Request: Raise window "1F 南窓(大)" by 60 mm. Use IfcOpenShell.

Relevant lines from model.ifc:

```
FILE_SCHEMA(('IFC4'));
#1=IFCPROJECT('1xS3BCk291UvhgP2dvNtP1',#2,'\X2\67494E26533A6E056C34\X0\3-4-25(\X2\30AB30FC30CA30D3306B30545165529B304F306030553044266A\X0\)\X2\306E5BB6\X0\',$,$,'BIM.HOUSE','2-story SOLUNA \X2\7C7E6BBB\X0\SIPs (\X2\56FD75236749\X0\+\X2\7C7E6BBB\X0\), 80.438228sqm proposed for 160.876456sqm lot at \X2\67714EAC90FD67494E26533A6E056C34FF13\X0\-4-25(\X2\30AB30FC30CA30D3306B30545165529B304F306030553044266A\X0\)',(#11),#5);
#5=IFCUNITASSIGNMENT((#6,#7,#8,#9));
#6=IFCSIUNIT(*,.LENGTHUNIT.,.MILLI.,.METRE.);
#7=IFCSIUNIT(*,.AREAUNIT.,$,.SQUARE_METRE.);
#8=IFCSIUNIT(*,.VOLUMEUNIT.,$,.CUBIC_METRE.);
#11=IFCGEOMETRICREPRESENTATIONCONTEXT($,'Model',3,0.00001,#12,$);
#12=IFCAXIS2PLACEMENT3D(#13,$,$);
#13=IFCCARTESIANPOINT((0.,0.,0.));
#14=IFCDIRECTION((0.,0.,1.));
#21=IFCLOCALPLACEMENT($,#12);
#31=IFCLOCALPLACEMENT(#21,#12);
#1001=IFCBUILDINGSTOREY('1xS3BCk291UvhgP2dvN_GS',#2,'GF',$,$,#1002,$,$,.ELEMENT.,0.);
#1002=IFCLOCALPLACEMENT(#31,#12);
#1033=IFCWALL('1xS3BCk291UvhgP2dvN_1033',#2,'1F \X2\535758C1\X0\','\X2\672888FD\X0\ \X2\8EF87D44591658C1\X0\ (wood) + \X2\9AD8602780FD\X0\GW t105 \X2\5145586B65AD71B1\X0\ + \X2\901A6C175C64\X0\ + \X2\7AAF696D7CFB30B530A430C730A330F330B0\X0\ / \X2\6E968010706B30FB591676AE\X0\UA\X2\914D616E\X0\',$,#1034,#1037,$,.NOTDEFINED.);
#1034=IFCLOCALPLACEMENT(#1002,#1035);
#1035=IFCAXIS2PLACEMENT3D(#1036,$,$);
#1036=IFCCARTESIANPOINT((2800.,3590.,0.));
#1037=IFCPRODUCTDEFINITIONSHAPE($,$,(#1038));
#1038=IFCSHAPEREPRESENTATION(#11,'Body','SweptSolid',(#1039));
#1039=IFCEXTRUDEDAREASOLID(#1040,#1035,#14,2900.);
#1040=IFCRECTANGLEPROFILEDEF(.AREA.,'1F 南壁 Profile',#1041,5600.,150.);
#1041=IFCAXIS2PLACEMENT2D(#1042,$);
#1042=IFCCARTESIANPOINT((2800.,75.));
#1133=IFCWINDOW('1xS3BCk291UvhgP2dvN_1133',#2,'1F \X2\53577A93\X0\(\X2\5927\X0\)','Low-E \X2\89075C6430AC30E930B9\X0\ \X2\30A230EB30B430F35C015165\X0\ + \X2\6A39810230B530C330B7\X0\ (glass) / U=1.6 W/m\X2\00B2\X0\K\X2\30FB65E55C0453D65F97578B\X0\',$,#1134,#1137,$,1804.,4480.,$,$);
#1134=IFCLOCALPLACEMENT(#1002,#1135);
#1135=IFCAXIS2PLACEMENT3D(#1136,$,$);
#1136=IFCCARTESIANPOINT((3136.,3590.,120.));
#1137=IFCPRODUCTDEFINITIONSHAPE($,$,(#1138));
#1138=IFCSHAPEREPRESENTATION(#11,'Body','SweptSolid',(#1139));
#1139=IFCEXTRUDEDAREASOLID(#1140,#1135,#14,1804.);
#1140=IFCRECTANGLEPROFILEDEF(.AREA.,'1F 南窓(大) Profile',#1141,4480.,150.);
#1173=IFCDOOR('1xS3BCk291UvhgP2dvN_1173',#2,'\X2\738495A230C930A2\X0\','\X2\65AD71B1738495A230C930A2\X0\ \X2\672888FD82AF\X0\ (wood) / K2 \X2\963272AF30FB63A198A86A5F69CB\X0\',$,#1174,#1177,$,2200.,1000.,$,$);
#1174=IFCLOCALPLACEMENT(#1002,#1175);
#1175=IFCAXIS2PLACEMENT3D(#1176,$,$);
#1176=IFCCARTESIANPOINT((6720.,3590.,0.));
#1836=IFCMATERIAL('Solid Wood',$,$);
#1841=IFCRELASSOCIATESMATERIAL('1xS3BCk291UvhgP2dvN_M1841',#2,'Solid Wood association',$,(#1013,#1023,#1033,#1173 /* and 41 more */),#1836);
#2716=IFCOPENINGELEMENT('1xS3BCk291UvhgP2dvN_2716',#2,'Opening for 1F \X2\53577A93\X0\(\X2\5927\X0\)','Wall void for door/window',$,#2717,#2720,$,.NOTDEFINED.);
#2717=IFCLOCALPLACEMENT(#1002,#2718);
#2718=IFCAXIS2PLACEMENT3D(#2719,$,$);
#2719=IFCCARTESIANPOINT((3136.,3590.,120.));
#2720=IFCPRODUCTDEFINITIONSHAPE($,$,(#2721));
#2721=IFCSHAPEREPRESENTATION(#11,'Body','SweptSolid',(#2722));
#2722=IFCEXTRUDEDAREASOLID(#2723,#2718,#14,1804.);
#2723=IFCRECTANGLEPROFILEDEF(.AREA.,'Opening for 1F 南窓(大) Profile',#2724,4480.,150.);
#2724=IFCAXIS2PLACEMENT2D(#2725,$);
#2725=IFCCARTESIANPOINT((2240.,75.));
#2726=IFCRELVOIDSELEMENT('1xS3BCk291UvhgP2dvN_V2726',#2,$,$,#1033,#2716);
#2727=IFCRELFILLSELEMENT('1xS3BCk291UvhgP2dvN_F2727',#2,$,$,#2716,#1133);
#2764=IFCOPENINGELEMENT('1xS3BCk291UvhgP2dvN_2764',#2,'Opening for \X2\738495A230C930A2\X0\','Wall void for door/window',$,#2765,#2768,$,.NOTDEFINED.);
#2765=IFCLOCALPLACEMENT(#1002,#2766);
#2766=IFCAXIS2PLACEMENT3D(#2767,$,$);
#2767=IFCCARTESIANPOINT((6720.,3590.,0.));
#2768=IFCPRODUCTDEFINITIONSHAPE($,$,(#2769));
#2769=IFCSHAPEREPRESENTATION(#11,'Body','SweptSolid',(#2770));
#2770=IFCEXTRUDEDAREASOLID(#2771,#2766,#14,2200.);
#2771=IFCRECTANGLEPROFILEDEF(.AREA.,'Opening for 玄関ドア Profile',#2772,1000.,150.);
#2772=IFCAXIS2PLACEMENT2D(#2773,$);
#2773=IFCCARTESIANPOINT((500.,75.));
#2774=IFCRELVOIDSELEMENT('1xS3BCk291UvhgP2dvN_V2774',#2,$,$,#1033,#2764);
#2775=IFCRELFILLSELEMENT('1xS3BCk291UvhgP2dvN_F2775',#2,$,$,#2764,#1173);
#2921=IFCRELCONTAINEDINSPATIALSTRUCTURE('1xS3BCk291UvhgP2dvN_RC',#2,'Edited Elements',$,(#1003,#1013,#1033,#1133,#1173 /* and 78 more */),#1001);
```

```python
import numpy as np
import ifcopenshell
import ifcopenshell.api.geometry
import ifcopenshell.util.placement
import ifcopenshell.util.unit

model = ifcopenshell.open("model.ifc")
unit_scale = ifcopenshell.util.unit.calculate_unit_scale(model)

window = model.by_guid("1xS3BCk291UvhgP2dvN_1133")
opening = window.FillsVoids[0].RelatingOpeningElement
dz = 60.0

shift = np.array([0.0, 0.0, dz])
# The window is not placed relative to its opening, so move both.
for product in (opening, window):
    matrix = ifcopenshell.util.placement.get_local_placement(product.ObjectPlacement)
    matrix[:3, 3] += shift
    ifcopenshell.api.geometry.edit_object_placement(model, product=product, matrix=matrix, is_si=False)

print(f"moved by {dz * unit_scale:+.3f} m")

model.write("model_updated.ifc")
```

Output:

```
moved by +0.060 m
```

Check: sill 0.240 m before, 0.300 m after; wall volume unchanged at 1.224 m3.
